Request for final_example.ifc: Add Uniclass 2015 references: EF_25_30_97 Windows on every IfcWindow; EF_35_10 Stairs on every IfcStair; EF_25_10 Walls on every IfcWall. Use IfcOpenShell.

First a look at what the model holds.

```python
import ifcopenshell

model = ifcopenshell.open("final_example.ifc")
print(model.schema)
print("classifications:", [c.Name for c in model.by_type("IfcClassification")])
for ifc_class in ("IfcDoor", "IfcRoof", "IfcStair", "IfcWall", "IfcWindow"):
    print(ifc_class, len(model.by_type(ifc_class)))
```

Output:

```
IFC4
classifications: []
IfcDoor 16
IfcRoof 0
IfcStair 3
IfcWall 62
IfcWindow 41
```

```python
import ifcopenshell
import ifcopenshell.api.classification

model = ifcopenshell.open("final_example.ifc")

system = ifcopenshell.api.classification.add_classification(model, classification="Uniclass 2015")

codes = {
    "IfcWindow": ("EF_25_30_97", "Windows"),
    "IfcStair": ("EF_35_10", "Stairs"),
    "IfcWall": ("EF_25_10", "Walls"),
}
for ifc_class, (code, name) in codes.items():
    products = model.by_type(ifc_class)
    ifcopenshell.api.classification.add_reference(
        model, products=products, classification=system, identification=code, name=name
    )
    print(code, len(products))

model.write("final_example_v2.ifc")
```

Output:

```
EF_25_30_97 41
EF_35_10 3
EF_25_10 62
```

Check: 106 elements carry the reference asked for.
